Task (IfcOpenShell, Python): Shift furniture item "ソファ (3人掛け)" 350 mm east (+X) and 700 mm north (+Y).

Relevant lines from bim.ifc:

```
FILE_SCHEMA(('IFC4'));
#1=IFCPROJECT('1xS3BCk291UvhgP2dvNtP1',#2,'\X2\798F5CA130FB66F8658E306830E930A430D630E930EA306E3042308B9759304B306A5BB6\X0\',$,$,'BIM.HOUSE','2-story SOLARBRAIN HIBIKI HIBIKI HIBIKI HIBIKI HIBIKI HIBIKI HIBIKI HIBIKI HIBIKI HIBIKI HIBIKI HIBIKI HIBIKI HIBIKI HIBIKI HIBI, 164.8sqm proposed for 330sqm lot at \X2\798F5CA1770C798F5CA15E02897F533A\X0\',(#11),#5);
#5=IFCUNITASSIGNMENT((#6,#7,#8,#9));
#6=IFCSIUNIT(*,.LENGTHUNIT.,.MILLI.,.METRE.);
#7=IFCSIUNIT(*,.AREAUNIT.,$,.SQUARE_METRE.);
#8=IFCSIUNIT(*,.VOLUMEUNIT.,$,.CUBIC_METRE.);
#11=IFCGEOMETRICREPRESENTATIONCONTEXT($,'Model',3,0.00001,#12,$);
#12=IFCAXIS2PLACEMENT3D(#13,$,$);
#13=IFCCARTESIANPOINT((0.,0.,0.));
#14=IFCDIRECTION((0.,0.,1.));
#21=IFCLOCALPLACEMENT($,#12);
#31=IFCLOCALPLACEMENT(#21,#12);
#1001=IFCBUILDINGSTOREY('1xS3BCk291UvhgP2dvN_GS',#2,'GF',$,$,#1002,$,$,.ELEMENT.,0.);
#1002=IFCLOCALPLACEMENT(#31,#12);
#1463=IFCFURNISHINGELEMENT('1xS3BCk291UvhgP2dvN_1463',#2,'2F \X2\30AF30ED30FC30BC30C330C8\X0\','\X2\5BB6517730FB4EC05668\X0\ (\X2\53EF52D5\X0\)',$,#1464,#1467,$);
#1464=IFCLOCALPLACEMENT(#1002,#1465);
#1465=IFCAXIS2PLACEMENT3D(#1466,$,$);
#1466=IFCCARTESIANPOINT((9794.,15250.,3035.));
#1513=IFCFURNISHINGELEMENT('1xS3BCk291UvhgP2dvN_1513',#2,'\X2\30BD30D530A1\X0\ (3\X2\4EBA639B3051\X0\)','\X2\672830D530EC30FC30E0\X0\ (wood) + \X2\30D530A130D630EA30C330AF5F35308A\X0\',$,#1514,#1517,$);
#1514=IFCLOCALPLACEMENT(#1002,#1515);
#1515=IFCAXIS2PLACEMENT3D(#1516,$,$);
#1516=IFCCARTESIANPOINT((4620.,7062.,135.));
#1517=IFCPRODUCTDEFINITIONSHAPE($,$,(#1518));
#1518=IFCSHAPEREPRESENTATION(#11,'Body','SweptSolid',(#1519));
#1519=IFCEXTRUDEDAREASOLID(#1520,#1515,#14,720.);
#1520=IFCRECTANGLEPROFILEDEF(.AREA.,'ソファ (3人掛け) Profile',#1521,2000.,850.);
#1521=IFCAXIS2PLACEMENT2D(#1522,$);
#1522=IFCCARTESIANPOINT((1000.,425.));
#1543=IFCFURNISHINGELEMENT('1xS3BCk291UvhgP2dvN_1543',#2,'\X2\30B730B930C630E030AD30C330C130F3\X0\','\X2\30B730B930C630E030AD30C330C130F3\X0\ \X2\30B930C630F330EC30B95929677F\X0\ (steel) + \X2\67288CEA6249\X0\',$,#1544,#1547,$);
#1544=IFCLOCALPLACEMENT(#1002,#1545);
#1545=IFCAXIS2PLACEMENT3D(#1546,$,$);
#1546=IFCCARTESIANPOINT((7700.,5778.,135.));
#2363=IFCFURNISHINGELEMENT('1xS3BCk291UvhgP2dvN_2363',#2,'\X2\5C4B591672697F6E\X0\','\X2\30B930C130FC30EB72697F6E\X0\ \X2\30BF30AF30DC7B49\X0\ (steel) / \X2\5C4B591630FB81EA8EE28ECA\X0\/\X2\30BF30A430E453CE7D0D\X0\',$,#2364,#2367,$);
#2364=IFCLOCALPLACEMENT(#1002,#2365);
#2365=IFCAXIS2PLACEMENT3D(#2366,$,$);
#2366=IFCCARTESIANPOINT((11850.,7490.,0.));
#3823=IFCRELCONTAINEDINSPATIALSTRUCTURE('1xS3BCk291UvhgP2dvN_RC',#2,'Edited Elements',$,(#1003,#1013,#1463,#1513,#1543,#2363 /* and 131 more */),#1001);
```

```python
import ifcopenshell
import ifcopenshell.api.geometry
import ifcopenshell.util.placement
import ifcopenshell.util.unit

model = ifcopenshell.open("bim.ifc")
unit_scale = ifcopenshell.util.unit.calculate_unit_scale(model)

item = model.by_guid("1xS3BCk291UvhgP2dvN_1513")
matrix = ifcopenshell.util.placement.get_local_placement(item.ObjectPlacement)
matrix[0, 3] += 0.35 / unit_scale
matrix[1, 3] += 0.7 / unit_scale
ifcopenshell.api.geometry.edit_object_placement(model, product=item, matrix=matrix, is_si=False)

print(ifcopenshell.util.placement.get_local_placement(item.ObjectPlacement).round(3) + 0.0)

model.write("bim-out.ifc")
```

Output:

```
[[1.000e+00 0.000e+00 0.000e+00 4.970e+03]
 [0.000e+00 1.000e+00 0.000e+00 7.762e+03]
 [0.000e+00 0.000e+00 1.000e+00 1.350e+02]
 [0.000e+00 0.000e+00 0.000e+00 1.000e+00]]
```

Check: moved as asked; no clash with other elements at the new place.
